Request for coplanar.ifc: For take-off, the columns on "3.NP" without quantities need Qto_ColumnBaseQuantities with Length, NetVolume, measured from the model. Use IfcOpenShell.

First a look at what the model holds.

```python
import ifcopenshell
import ifcopenshell.util.element
import ifcopenshell.util.unit

model = ifcopenshell.open("coplanar.ifc")
print(model.schema)
for unit_type in ("LENGTHUNIT", "AREAUNIT", "VOLUMEUNIT"):
    print(unit_type, ifcopenshell.util.unit.calculate_unit_scale(model, unit_type))
storey = next(s for s in model.by_type("IfcBuildingStorey") if s.Name == "3.NP")
columns = [e for e in ifcopenshell.util.element.get_decomposition(storey) if e.is_a("IfcColumn")]
for e in sorted(columns, key=lambda e: e.id()):
    print(e.id(), e.is_a(), e.Name, list(ifcopenshell.util.element.get_psets(e, qtos_only=True)), sep=" | ")
```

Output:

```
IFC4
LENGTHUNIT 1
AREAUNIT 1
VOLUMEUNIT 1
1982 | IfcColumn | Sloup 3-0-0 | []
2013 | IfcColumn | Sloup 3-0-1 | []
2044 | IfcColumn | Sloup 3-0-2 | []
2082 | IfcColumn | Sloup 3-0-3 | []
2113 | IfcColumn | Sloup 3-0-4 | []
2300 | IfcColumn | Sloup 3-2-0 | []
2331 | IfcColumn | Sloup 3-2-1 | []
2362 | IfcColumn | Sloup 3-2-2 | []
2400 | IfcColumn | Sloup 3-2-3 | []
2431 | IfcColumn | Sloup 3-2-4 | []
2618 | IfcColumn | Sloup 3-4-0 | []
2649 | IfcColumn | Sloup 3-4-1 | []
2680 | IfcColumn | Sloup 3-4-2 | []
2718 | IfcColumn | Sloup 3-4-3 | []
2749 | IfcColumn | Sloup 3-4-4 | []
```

```python
import ifcopenshell
import ifcopenshell.api.pset
import ifcopenshell.geom
import ifcopenshell.util.element
import ifcopenshell.util.shape
import ifcopenshell.util.unit

model = ifcopenshell.open("coplanar.ifc")
unit_scale = ifcopenshell.util.unit.calculate_unit_scale(model)
volume_scale = ifcopenshell.util.unit.calculate_unit_scale(model, "VOLUMEUNIT")
settings = ifcopenshell.geom.settings()

storey = next(s for s in model.by_type("IfcBuildingStorey") if s.Name == "3.NP")
columns = [e for e in ifcopenshell.util.element.get_decomposition(storey) if e.is_a("IfcColumn")]

for e in sorted(columns, key=lambda e: e.id()):
    if ifcopenshell.util.element.get_psets(e, qtos_only=True, should_inherit=False):
        continue
    # Geometry comes back in metres, in the element's own axes.
    shape = ifcopenshell.geom.create_shape(settings, e)
    values = {
        "Length": ifcopenshell.util.shape.get_z(shape.geometry) / unit_scale,
        "NetVolume": ifcopenshell.util.shape.get_volume(shape.geometry) / volume_scale,
    }
    qto = ifcopenshell.api.pset.add_qto(model, product=e, name="Qto_ColumnBaseQuantities")
    ifcopenshell.api.pset.edit_qto(model, qto=qto, properties=values)
    print(e.id(), {k: round(v, 3) for k, v in values.items()})

model.write("coplanar_edited.ifc")
```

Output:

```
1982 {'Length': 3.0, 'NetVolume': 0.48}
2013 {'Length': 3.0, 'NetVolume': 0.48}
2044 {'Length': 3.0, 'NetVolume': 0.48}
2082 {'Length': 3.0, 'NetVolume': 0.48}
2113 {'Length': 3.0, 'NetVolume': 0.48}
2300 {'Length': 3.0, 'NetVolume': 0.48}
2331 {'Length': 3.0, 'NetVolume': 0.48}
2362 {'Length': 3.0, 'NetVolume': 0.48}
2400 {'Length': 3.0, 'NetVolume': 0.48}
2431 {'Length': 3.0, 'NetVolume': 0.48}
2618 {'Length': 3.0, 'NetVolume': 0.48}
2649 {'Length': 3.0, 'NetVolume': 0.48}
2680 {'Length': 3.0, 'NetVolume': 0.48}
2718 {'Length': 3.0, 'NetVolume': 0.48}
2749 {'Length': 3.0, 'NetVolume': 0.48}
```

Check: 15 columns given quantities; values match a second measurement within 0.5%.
